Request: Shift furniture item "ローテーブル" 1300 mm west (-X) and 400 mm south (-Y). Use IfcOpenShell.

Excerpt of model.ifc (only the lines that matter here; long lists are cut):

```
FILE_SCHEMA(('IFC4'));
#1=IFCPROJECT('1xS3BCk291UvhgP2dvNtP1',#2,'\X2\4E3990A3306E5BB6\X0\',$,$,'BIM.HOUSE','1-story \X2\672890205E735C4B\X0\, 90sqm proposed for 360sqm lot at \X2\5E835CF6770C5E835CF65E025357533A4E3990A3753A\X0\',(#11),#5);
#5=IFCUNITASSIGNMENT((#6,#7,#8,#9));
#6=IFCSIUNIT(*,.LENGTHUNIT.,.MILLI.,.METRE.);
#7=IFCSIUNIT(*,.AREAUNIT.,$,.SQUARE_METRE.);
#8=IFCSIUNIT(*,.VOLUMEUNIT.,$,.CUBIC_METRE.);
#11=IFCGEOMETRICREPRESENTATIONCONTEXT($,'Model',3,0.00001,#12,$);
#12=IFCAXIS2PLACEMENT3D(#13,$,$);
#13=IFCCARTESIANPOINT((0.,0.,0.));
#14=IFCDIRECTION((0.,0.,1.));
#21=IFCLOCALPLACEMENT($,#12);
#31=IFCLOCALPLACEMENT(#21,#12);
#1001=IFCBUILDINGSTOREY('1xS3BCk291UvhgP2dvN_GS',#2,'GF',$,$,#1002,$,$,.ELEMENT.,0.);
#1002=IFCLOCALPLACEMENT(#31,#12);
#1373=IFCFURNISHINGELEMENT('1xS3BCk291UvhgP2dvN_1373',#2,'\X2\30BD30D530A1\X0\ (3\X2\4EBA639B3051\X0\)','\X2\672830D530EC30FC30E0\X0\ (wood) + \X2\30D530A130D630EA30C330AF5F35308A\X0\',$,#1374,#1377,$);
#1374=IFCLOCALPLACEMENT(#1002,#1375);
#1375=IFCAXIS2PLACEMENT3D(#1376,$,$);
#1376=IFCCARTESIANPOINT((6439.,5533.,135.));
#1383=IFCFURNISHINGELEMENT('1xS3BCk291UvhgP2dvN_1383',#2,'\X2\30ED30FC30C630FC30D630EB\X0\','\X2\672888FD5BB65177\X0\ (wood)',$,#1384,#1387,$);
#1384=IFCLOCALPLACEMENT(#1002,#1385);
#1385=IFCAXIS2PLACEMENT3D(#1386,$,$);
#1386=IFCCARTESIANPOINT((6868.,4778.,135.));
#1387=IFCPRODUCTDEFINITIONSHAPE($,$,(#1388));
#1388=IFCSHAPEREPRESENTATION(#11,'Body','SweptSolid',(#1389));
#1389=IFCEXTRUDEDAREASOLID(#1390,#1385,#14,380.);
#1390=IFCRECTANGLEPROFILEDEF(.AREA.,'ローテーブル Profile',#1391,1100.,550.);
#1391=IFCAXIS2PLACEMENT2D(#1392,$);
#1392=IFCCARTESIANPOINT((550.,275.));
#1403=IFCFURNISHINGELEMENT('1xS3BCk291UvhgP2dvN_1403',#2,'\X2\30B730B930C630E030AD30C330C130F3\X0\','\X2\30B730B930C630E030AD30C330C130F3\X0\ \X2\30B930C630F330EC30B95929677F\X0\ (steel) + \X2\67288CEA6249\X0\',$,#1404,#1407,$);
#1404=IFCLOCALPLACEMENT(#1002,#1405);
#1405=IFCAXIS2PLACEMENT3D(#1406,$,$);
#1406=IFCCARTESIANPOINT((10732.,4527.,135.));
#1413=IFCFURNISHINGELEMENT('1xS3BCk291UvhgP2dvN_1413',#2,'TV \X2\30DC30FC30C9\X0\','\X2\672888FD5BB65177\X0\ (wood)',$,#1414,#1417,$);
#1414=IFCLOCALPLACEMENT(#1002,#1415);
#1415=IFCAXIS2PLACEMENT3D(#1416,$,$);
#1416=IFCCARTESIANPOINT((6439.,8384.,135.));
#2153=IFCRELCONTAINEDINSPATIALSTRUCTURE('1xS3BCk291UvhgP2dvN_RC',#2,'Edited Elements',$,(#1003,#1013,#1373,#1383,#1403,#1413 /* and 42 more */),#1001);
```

```python
import ifcopenshell
import ifcopenshell.api.geometry
import ifcopenshell.util.placement
import ifcopenshell.util.unit

model = ifcopenshell.open("model.ifc")
unit_scale = ifcopenshell.util.unit.calculate_unit_scale(model)

item = model.by_id(1383)
matrix = ifcopenshell.util.placement.get_local_placement(item.ObjectPlacement)
matrix[0, 3] -= 1.3 / unit_scale
matrix[1, 3] -= 0.4 / unit_scale
ifcopenshell.api.geometry.edit_object_placement(model, product=item, matrix=matrix, is_si=False)

print(ifcopenshell.util.placement.get_local_placement(item.ObjectPlacement).round(3) + 0.0)

model.write("model-out.ifc")
```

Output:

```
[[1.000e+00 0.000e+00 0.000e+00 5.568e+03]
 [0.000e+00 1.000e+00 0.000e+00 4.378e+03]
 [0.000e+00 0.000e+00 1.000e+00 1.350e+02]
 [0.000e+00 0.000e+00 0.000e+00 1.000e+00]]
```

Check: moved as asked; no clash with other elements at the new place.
